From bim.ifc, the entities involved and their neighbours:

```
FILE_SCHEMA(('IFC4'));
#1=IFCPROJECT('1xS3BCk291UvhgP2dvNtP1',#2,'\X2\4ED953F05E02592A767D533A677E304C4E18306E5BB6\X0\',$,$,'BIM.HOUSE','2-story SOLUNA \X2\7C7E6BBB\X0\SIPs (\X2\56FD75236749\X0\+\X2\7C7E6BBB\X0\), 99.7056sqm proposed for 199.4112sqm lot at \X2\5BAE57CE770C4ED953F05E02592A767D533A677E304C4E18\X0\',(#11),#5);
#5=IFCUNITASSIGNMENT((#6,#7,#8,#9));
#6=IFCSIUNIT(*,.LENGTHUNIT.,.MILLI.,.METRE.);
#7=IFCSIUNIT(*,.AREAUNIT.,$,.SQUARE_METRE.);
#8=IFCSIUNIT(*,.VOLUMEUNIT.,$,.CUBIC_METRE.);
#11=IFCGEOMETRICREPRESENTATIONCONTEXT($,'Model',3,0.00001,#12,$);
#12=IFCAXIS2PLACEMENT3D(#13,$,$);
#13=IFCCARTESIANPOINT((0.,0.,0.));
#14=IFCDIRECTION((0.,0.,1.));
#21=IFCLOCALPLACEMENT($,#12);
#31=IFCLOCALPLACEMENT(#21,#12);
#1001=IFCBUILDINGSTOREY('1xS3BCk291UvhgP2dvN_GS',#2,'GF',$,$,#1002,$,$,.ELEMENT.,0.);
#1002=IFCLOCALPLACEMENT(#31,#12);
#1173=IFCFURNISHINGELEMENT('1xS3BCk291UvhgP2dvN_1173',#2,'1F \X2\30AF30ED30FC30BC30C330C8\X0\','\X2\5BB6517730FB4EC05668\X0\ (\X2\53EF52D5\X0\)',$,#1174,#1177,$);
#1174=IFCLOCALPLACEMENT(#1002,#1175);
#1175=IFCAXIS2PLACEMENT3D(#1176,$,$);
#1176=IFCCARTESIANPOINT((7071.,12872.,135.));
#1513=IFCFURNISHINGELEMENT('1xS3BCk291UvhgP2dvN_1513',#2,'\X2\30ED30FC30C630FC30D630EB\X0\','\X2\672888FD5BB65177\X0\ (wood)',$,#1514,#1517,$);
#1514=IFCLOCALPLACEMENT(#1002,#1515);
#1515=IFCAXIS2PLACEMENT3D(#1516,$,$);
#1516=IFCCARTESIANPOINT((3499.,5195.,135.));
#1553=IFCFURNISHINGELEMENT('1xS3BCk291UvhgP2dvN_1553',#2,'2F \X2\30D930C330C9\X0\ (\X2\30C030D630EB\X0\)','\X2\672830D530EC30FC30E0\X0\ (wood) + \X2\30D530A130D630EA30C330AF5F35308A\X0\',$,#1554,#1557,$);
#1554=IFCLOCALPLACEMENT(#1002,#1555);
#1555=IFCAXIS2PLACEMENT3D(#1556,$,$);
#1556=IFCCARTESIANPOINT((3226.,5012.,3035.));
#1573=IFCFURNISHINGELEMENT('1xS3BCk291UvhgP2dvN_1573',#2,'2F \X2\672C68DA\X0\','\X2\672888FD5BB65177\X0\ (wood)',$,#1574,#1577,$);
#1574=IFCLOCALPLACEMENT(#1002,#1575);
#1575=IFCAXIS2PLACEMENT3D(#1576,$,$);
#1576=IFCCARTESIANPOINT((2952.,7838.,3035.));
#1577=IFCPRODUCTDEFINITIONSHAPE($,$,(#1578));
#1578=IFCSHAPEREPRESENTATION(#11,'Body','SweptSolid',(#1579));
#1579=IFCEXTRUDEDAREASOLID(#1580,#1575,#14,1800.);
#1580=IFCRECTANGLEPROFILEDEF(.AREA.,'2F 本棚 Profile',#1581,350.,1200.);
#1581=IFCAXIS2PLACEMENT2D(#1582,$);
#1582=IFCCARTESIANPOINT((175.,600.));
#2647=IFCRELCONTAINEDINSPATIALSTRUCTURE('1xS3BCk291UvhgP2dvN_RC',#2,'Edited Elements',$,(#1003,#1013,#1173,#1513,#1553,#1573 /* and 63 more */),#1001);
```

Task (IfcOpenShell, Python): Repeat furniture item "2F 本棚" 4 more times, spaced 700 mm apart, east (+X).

```python
import numpy as np
import ifcopenshell
import ifcopenshell.api.geometry
import ifcopenshell.api.root
import ifcopenshell.util.element
import ifcopenshell.util.placement
import ifcopenshell.util.unit

model = ifcopenshell.open("bim.ifc")
unit_scale = ifcopenshell.util.unit.calculate_unit_scale(model)


def reuse_history(source, copy):
    """copy_class also copies each property set's owner history, people and application; keep the originals."""
    for rel in copy.IsDefinedBy:
        if rel.is_a("IfcRelDefinesByProperties") and (history := rel.RelatingPropertyDefinition.OwnerHistory):
            rel.RelatingPropertyDefinition.OwnerHistory = source.OwnerHistory
            ifcopenshell.util.element.remove_deep2(model, history)


source = model.by_guid("1xS3BCk291UvhgP2dvN_1573")
base = ifcopenshell.util.placement.get_local_placement(source.ObjectPlacement)
step = np.array([1.0, 0.0, 0.0]) * 0.7 / unit_scale

for i in range(1, 5):
    copy = ifcopenshell.api.root.copy_class(model, product=source)
    copy.Representation = ifcopenshell.util.element.copy_deep(
        model, source.Representation, exclude=["IfcGeometricRepresentationContext", "IfcRepresentationMap"]
    )
    reuse_history(source, copy)
    matrix = base.copy()
    matrix[:3, 3] += i * step
    print("added at", matrix[:3, 3].round(3) + 0.0)
    ifcopenshell.api.geometry.edit_object_placement(model, product=copy, matrix=matrix, is_si=False)

model.write("bim_edited.ifc")
```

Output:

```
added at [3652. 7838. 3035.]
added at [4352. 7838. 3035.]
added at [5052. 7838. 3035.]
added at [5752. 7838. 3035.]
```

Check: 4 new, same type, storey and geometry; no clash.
